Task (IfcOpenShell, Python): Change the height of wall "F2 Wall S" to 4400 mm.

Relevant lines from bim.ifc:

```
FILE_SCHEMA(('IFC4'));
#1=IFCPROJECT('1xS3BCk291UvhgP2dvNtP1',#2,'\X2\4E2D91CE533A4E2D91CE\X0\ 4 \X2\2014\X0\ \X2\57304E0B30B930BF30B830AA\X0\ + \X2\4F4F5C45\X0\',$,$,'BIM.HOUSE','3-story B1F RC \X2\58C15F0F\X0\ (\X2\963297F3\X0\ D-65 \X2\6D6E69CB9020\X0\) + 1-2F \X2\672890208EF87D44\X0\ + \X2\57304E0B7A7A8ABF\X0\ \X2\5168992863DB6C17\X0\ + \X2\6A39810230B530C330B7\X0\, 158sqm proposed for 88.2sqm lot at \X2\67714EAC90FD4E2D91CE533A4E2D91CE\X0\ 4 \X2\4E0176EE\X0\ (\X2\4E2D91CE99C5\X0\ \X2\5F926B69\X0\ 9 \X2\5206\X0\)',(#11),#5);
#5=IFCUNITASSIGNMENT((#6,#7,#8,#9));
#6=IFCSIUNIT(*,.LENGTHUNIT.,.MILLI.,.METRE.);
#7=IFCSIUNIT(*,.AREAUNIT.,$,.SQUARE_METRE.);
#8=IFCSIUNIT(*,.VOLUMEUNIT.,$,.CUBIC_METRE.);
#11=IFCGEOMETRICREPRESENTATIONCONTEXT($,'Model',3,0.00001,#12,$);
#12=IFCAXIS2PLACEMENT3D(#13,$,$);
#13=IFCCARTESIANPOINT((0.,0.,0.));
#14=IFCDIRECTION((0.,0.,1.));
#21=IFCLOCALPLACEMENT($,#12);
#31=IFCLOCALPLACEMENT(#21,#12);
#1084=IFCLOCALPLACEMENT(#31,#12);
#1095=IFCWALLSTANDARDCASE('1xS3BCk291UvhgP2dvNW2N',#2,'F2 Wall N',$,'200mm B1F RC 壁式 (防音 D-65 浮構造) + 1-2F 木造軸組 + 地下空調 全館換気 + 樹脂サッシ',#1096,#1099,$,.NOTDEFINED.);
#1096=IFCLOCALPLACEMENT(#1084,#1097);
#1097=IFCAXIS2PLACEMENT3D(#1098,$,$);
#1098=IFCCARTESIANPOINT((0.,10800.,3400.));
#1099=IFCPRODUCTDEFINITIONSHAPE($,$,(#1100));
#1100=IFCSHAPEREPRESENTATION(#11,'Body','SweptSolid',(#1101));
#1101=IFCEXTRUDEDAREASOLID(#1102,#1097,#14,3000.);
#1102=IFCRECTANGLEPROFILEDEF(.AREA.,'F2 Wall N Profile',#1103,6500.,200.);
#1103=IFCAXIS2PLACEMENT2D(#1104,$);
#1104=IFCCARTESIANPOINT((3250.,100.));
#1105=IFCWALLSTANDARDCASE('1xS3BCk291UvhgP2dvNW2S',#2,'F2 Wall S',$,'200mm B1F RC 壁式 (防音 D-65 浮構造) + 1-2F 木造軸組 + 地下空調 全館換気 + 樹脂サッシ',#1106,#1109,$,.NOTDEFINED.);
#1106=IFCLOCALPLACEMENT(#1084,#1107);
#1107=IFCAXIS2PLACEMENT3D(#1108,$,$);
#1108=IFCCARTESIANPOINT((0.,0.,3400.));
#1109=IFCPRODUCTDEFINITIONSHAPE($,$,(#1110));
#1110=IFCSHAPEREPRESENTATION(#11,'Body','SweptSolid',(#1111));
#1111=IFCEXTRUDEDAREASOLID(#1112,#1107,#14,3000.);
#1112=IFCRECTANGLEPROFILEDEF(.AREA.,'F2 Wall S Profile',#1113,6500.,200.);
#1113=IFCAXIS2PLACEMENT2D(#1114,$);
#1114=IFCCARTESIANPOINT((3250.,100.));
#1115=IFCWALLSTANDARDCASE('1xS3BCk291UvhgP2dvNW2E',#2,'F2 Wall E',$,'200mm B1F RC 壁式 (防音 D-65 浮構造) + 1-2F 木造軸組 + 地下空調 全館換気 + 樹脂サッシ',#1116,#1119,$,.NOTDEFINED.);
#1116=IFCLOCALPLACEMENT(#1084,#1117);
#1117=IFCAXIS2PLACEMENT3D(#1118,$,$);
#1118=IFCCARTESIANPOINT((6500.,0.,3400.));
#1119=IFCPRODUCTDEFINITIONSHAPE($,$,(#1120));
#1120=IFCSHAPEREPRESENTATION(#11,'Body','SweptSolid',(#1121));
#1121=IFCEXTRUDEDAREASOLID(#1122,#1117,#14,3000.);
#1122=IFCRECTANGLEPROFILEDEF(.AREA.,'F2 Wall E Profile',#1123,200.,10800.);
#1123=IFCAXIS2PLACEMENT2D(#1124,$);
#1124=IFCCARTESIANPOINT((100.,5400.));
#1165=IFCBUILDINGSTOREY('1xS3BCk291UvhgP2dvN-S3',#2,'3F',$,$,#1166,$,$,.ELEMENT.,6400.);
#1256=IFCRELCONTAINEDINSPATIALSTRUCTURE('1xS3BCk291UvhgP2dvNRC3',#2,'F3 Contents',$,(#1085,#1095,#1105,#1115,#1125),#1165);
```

```python
import ifcopenshell
import ifcopenshell.geom
import ifcopenshell.util.shape

model = ifcopenshell.open("bim.ifc")
settings = ifcopenshell.geom.settings()


def volume(element):
    """Net volume in cubic metres, openings subtracted."""
    shape = ifcopenshell.geom.create_shape(settings, element)
    return ifcopenshell.util.shape.get_volume(shape.geometry)


wall = model.by_id(1105)
before = volume(wall)

body = next(r for r in wall.Representation.Representations if r.RepresentationIdentifier == "Body")
solid = body.Items[0]
old_height = solid.Depth
solid.Depth = 4400.0
after = volume(wall)

print(f"height {old_height:g} -> {solid.Depth:g}, volume {before:.3f} -> {after:.3f} m3")

model.write("bim-out.ifc")
```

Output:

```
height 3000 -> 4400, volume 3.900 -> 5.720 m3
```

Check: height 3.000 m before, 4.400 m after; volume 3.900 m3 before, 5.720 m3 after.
